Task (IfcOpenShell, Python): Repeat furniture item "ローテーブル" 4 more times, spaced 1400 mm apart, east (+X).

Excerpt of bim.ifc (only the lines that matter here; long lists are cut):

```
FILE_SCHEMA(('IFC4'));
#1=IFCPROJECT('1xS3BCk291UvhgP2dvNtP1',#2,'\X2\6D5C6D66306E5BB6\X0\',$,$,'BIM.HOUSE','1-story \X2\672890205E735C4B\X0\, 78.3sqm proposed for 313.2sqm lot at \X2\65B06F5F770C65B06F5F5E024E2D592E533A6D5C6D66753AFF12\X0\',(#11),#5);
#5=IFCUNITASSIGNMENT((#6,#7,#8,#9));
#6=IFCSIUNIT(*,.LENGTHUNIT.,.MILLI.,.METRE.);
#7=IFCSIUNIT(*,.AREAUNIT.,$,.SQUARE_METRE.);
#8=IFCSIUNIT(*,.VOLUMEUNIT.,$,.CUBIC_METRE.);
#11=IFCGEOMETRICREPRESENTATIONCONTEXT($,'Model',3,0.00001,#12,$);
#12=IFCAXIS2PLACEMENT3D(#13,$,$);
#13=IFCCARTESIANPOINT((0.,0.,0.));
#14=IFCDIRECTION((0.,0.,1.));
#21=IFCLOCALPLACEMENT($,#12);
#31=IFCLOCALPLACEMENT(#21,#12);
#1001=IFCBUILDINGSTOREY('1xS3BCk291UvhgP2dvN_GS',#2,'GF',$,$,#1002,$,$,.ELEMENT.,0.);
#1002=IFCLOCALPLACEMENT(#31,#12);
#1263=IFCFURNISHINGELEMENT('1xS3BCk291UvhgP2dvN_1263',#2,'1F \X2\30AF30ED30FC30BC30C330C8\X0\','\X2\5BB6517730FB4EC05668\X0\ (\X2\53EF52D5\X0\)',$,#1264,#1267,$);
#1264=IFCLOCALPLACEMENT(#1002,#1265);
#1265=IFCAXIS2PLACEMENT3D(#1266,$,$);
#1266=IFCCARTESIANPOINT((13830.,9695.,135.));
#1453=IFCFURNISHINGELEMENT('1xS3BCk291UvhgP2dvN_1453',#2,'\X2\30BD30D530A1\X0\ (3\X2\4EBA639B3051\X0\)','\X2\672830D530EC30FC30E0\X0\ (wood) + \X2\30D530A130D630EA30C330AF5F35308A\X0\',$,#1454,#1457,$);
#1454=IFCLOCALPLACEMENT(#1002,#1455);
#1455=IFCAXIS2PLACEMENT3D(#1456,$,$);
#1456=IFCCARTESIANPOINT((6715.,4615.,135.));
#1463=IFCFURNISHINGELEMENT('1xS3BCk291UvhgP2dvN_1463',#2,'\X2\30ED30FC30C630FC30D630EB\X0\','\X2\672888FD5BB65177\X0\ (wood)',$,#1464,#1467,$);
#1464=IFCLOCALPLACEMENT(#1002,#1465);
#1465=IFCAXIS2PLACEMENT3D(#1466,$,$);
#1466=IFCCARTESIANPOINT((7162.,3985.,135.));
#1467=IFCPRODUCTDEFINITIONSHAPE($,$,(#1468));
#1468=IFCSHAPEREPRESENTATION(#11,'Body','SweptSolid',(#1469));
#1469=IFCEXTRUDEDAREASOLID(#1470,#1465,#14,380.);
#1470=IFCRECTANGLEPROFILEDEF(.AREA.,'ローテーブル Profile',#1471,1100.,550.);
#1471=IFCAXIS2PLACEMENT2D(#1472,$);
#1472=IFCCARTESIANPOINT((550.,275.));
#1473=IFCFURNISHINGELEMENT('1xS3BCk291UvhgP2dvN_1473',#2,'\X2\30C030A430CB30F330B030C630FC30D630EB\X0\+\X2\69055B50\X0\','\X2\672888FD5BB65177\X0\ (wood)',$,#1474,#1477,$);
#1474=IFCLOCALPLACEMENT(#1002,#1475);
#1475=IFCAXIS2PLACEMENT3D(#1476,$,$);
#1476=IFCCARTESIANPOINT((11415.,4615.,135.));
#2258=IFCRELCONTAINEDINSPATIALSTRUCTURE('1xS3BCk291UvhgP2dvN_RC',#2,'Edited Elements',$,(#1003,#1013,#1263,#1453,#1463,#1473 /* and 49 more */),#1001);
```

```python
import numpy as np
import ifcopenshell
import ifcopenshell.api.geometry
import ifcopenshell.api.root
import ifcopenshell.util.element
import ifcopenshell.util.placement
import ifcopenshell.util.unit

model = ifcopenshell.open("bim.ifc")
unit_scale = ifcopenshell.util.unit.calculate_unit_scale(model)


def reuse_history(source, copy):
    """copy_class also copies each property set's owner history, people and application; keep the originals."""
    for rel in copy.IsDefinedBy:
        if rel.is_a("IfcRelDefinesByProperties") and (history := rel.RelatingPropertyDefinition.OwnerHistory):
            rel.RelatingPropertyDefinition.OwnerHistory = source.OwnerHistory
            ifcopenshell.util.element.remove_deep2(model, history)


source = model.by_guid("1xS3BCk291UvhgP2dvN_1463")
base = ifcopenshell.util.placement.get_local_placement(source.ObjectPlacement)
step = np.array([1.0, 0.0, 0.0]) * 1.4 / unit_scale

for i in range(1, 5):
    copy = ifcopenshell.api.root.copy_class(model, product=source)
    copy.Representation = ifcopenshell.util.element.copy_deep(
        model, source.Representation, exclude=["IfcGeometricRepresentationContext", "IfcRepresentationMap"]
    )
    reuse_history(source, copy)
    matrix = base.copy()
    matrix[:3, 3] += i * step
    print("added at", matrix[:3, 3].round(3) + 0.0)
    ifcopenshell.api.geometry.edit_object_placement(model, product=copy, matrix=matrix, is_si=False)

model.write("bim_v2.ifc")
```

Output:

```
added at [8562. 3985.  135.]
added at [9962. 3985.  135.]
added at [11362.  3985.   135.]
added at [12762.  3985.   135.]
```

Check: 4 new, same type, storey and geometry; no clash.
